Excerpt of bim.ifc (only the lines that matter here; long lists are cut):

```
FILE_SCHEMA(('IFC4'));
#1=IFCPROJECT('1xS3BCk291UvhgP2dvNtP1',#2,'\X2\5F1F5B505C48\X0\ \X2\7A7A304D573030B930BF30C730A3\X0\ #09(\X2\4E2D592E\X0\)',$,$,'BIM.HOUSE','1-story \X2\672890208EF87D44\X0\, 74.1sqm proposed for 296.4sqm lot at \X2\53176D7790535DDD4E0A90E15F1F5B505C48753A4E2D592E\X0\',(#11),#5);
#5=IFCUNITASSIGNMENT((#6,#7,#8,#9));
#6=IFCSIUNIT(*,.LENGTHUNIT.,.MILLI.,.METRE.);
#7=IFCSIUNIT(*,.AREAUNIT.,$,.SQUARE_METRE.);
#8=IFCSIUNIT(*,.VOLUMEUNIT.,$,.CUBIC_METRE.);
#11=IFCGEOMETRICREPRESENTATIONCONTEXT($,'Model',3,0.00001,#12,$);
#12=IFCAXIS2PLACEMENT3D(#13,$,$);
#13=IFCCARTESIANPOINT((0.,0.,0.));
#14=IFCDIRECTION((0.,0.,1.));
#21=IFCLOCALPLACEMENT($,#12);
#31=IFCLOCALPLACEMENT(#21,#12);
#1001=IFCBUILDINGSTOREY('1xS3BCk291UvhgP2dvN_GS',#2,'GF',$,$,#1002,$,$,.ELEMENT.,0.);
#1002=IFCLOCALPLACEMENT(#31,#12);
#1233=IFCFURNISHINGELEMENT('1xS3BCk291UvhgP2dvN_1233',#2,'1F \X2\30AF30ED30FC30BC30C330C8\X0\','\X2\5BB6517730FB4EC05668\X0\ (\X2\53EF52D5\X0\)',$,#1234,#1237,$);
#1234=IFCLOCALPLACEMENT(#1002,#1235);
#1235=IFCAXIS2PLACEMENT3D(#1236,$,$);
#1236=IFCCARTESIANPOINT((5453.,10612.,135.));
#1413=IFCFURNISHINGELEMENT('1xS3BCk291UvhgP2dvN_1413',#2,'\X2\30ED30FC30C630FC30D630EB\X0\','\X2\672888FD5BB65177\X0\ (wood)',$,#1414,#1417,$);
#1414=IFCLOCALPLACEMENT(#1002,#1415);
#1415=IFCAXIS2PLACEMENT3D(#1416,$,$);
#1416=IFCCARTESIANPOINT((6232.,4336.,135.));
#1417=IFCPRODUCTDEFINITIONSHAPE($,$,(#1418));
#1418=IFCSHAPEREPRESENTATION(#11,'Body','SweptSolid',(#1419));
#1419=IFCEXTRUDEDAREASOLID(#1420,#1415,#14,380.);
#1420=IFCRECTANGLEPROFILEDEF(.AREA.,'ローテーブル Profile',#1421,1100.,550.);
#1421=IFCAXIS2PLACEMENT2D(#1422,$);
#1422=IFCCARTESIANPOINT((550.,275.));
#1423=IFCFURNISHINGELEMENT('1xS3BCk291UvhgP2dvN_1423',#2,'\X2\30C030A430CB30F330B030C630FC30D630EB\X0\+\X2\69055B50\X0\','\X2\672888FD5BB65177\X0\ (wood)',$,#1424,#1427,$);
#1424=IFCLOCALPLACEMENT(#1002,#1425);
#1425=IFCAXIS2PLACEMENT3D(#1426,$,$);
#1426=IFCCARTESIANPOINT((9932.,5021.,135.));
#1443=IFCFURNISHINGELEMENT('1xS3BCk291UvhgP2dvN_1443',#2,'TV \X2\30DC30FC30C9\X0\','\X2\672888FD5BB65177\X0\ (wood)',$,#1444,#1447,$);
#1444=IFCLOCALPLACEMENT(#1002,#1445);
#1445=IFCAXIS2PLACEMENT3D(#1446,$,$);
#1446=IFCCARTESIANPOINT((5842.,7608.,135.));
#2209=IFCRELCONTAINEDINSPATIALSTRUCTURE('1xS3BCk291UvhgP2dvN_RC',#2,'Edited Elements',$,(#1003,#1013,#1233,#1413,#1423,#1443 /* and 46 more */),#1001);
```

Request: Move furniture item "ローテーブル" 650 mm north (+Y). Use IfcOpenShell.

```python
import ifcopenshell
import ifcopenshell.api.geometry
import ifcopenshell.util.placement
import ifcopenshell.util.unit

model = ifcopenshell.open("bim.ifc")
unit_scale = ifcopenshell.util.unit.calculate_unit_scale(model)

item = model.by_guid("1xS3BCk291UvhgP2dvN_1413")
matrix = ifcopenshell.util.placement.get_local_placement(item.ObjectPlacement)
matrix[1, 3] += 0.65 / unit_scale
ifcopenshell.api.geometry.edit_object_placement(model, product=item, matrix=matrix, is_si=False)

print(ifcopenshell.util.placement.get_local_placement(item.ObjectPlacement).round(3) + 0.0)

model.write("bim_edited.ifc")
```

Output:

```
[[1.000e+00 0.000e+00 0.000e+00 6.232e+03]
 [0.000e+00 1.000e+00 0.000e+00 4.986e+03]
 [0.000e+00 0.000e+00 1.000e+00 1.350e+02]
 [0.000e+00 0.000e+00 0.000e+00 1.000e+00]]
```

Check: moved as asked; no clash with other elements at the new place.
